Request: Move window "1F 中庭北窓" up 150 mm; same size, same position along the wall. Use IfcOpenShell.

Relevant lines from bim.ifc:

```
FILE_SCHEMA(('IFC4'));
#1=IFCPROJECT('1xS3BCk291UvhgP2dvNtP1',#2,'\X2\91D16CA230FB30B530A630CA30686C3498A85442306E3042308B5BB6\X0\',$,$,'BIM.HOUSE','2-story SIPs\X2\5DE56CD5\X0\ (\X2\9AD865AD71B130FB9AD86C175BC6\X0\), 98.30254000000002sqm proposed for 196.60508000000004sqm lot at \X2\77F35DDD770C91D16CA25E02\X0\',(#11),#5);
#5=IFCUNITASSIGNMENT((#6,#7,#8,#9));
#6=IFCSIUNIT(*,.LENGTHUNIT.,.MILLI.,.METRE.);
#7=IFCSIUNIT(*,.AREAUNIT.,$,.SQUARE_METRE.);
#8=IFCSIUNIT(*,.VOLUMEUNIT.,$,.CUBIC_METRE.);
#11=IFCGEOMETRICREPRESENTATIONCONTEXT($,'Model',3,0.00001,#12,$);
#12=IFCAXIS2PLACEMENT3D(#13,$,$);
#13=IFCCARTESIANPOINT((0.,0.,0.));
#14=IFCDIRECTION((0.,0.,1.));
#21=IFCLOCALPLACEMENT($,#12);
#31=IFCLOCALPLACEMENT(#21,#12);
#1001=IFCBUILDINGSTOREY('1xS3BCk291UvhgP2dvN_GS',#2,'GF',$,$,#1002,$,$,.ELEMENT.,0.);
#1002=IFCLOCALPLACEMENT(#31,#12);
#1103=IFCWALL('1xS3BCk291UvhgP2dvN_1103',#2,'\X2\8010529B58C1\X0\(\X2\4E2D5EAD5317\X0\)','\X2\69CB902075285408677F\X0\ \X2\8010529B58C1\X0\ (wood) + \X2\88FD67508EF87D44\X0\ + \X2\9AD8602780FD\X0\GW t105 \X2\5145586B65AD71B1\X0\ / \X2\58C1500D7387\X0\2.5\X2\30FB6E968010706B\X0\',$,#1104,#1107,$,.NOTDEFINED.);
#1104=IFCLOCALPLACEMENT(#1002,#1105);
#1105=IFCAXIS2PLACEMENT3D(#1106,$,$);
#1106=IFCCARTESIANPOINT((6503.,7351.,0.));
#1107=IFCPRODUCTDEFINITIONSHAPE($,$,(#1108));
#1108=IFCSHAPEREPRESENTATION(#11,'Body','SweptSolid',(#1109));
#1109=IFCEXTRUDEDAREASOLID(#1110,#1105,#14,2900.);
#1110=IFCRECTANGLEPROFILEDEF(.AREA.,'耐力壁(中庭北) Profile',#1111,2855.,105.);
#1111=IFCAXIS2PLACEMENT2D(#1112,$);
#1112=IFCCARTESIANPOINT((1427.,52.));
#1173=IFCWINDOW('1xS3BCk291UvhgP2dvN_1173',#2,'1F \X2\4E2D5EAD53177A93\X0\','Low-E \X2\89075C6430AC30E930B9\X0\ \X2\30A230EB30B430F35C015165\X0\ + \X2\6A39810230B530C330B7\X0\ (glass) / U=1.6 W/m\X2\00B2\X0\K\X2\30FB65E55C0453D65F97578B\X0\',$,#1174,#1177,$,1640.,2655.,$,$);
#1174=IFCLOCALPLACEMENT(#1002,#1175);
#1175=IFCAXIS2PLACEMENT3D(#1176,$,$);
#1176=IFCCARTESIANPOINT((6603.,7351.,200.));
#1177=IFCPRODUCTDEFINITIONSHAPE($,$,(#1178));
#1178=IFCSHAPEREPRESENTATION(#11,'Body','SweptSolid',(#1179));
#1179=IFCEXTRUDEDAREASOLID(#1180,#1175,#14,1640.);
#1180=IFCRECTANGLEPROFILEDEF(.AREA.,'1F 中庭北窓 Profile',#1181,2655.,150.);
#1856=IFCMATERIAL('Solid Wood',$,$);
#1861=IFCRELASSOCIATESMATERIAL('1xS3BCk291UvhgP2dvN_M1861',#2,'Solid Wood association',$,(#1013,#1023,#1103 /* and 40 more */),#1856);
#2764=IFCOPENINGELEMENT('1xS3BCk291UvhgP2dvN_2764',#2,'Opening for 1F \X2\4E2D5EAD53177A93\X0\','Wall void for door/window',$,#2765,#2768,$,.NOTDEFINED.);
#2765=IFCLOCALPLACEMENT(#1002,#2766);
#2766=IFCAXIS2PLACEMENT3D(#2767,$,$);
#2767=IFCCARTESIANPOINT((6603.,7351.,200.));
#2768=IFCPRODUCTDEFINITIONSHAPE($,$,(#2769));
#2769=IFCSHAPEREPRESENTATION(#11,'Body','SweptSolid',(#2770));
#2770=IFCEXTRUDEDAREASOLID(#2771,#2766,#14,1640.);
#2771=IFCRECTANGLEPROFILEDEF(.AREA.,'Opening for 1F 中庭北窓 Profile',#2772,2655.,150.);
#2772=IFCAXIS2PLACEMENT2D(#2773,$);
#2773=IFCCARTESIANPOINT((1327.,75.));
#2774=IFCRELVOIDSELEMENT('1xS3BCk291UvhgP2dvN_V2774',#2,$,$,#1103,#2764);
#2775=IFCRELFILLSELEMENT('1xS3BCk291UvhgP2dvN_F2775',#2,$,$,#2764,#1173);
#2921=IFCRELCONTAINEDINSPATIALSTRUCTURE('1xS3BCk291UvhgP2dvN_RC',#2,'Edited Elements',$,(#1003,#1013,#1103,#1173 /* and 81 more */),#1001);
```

```python
import numpy as np
import ifcopenshell
import ifcopenshell.api.geometry
import ifcopenshell.util.placement
import ifcopenshell.util.unit

model = ifcopenshell.open("bim.ifc")
unit_scale = ifcopenshell.util.unit.calculate_unit_scale(model)

window = model.by_guid("1xS3BCk291UvhgP2dvN_1173")
opening = window.FillsVoids[0].RelatingOpeningElement
dz = 0.15 / unit_scale

shift = np.array([0.0, 0.0, dz])
# The window is not placed relative to its opening, so move both.
for product in (opening, window):
    matrix = ifcopenshell.util.placement.get_local_placement(product.ObjectPlacement)
    matrix[:3, 3] += shift
    ifcopenshell.api.geometry.edit_object_placement(model, product=product, matrix=matrix, is_si=False)

print(f"moved by {dz * unit_scale:+.3f} m")

model.write("bim_v2.ifc")
```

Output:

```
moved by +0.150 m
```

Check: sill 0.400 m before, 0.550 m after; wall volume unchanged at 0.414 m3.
